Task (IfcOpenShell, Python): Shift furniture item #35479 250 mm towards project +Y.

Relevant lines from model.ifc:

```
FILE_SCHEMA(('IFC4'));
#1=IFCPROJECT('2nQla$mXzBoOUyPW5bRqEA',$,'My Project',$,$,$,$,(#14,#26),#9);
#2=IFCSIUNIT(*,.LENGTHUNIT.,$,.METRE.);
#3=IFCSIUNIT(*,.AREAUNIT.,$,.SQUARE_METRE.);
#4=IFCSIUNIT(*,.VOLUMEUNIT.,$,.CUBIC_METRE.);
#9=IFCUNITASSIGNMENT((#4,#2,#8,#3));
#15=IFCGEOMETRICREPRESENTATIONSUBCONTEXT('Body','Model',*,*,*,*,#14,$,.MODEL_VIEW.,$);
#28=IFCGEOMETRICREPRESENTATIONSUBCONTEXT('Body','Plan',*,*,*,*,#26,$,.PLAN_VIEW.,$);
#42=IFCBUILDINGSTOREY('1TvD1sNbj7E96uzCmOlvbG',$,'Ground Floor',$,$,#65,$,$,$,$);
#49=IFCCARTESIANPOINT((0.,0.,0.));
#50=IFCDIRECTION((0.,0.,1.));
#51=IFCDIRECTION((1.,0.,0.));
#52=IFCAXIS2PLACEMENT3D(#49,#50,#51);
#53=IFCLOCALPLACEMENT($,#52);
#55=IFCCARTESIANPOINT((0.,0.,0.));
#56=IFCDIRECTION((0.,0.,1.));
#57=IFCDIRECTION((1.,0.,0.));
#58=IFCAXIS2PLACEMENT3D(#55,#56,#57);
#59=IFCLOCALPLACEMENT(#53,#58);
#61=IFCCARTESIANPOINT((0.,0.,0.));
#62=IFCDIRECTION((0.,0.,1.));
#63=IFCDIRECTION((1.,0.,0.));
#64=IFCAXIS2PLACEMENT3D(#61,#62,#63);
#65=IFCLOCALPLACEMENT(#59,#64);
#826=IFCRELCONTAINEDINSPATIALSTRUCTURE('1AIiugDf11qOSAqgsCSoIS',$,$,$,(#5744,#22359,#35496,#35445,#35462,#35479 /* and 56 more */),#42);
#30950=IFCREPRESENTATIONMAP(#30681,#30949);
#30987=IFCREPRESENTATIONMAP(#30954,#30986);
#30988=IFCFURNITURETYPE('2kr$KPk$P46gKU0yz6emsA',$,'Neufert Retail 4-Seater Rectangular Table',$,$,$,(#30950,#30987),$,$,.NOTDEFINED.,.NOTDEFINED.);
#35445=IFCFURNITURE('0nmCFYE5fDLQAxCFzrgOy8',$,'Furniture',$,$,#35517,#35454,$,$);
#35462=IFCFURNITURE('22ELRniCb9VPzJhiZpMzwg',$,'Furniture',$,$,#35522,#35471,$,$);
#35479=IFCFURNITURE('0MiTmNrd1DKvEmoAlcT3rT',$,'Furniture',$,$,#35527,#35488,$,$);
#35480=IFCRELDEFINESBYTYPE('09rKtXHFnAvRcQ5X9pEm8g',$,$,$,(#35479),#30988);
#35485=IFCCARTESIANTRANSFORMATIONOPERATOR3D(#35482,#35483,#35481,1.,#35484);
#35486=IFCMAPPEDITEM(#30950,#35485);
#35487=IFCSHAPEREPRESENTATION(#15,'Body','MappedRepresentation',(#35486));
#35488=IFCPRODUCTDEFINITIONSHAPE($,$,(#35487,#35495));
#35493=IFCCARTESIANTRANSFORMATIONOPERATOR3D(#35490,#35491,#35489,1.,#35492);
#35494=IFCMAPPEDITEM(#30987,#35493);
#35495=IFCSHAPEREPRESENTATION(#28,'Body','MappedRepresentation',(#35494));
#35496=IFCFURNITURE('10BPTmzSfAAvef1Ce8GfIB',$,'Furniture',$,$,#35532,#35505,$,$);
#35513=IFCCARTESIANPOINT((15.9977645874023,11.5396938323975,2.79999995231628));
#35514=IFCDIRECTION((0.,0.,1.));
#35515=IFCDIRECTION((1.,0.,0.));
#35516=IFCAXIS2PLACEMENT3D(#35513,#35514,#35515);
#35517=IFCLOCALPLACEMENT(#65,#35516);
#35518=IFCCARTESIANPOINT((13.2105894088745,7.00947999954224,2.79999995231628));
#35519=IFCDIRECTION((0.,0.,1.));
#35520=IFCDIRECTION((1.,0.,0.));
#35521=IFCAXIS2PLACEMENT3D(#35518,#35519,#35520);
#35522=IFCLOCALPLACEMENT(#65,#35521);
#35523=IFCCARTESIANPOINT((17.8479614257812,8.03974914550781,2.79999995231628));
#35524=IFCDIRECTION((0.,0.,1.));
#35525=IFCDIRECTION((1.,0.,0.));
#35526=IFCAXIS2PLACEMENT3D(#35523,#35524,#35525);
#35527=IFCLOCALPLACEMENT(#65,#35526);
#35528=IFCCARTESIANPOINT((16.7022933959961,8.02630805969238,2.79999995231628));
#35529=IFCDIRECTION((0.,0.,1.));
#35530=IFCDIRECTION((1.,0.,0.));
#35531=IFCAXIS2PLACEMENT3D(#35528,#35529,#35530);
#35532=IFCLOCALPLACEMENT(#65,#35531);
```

```python
import ifcopenshell
import ifcopenshell.api.geometry
import ifcopenshell.util.placement

model = ifcopenshell.open("model.ifc")

item = model.by_guid("0MiTmNrd1DKvEmoAlcT3rT")
matrix = ifcopenshell.util.placement.get_local_placement(item.ObjectPlacement)
matrix[1, 3] += 0.25
ifcopenshell.api.geometry.edit_object_placement(model, product=item, matrix=matrix, is_si=False)

print(ifcopenshell.util.placement.get_local_placement(item.ObjectPlacement).round(3) + 0.0)

model.write("model-out.ifc")
```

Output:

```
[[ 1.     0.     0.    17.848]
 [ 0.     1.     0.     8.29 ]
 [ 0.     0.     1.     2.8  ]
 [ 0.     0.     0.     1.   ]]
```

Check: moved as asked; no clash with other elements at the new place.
